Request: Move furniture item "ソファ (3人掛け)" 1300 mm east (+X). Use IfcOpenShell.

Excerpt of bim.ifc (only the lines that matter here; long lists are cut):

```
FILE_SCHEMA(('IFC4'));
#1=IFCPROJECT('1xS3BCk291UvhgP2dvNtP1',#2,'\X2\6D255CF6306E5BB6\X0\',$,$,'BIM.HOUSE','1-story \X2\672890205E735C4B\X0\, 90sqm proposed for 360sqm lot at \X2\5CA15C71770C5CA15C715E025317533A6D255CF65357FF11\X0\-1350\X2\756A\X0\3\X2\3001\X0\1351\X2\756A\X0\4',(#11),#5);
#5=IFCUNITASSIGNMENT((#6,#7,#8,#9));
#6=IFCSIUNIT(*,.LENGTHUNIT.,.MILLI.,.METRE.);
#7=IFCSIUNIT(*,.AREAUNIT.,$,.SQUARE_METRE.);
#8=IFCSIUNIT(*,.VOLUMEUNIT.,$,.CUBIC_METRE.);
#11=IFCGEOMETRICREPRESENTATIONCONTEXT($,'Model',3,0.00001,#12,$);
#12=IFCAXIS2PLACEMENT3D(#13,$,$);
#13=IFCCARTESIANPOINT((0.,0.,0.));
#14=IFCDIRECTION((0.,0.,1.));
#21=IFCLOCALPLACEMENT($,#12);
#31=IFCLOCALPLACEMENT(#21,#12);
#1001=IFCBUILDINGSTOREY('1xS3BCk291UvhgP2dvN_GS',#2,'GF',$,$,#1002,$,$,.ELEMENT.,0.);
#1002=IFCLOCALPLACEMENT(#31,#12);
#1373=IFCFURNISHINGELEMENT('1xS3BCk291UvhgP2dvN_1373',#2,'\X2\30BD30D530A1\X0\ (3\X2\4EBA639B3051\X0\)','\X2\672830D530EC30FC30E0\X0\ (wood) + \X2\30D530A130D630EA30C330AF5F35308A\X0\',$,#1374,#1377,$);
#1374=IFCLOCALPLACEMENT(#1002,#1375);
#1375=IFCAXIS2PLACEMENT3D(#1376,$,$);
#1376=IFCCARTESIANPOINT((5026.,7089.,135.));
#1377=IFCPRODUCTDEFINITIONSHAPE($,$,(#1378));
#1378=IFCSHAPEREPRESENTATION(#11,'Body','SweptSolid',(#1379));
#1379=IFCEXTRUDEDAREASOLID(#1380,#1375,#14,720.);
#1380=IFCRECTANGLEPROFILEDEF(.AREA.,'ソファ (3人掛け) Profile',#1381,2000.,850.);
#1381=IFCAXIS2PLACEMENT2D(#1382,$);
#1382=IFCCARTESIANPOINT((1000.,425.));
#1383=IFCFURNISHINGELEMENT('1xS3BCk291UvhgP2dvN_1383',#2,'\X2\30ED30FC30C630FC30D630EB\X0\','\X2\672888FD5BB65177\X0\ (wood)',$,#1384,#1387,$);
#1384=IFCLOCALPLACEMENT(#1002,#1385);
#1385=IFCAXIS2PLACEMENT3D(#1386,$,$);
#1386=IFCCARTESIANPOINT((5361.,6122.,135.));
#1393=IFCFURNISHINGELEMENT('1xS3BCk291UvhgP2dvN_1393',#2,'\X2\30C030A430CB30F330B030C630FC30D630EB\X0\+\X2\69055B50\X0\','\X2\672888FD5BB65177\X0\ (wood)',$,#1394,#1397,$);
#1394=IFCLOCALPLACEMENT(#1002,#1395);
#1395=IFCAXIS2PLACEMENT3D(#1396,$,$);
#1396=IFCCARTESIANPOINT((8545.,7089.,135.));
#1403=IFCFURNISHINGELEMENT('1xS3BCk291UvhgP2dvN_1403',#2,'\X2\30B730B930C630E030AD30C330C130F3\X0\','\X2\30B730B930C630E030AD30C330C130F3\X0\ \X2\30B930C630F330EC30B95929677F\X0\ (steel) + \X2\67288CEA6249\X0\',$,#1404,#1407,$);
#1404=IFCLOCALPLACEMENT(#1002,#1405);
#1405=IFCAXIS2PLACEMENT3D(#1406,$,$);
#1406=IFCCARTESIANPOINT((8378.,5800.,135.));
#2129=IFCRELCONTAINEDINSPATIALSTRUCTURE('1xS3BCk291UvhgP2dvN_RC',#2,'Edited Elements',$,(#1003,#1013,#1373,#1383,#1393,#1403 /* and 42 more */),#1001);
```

```python
import ifcopenshell
import ifcopenshell.api.geometry
import ifcopenshell.util.placement
import ifcopenshell.util.unit

model = ifcopenshell.open("bim.ifc")
unit_scale = ifcopenshell.util.unit.calculate_unit_scale(model)

item = model.by_id(1373)
matrix = ifcopenshell.util.placement.get_local_placement(item.ObjectPlacement)
matrix[0, 3] += 1.3 / unit_scale
ifcopenshell.api.geometry.edit_object_placement(model, product=item, matrix=matrix, is_si=False)

print(ifcopenshell.util.placement.get_local_placement(item.ObjectPlacement).round(3) + 0.0)

model.write("bim_rev.ifc")
```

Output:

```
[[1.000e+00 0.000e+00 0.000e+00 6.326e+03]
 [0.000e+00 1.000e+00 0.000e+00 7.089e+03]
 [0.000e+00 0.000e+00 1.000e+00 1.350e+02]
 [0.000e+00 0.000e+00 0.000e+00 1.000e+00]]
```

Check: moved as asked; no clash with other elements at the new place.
